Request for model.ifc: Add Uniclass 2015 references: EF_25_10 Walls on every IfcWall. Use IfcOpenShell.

First a look at what the model holds.

```python
import ifcopenshell

model = ifcopenshell.open("model.ifc")
print(model.schema)
print("classifications:", [c.Name for c in model.by_type("IfcClassification")])
for ifc_class in ("IfcDoor", "IfcRoof", "IfcStair", "IfcWall", "IfcWindow"):
    print(ifc_class, len(model.by_type(ifc_class)))
```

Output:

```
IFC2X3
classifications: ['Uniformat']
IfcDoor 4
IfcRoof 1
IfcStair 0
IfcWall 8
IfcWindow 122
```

```python
import ifcopenshell
import ifcopenshell.api.classification

model = ifcopenshell.open("model.ifc")

# IFC2X3 requires Source and Edition and has no link from the project to the system.
system = model.create_entity("IfcClassification", Source="NBS", Edition="2015", Name="Uniclass 2015")

codes = {
    "IfcWall": ("EF_25_10", "Walls"),
}
for ifc_class, (code, name) in codes.items():
    products = model.by_type(ifc_class)
    ifcopenshell.api.classification.add_reference(
        model, products=products, classification=system, identification=code, name=name
    )
    print(code, len(products))

model.write("model_updated.ifc")
```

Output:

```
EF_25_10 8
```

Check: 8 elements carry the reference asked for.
